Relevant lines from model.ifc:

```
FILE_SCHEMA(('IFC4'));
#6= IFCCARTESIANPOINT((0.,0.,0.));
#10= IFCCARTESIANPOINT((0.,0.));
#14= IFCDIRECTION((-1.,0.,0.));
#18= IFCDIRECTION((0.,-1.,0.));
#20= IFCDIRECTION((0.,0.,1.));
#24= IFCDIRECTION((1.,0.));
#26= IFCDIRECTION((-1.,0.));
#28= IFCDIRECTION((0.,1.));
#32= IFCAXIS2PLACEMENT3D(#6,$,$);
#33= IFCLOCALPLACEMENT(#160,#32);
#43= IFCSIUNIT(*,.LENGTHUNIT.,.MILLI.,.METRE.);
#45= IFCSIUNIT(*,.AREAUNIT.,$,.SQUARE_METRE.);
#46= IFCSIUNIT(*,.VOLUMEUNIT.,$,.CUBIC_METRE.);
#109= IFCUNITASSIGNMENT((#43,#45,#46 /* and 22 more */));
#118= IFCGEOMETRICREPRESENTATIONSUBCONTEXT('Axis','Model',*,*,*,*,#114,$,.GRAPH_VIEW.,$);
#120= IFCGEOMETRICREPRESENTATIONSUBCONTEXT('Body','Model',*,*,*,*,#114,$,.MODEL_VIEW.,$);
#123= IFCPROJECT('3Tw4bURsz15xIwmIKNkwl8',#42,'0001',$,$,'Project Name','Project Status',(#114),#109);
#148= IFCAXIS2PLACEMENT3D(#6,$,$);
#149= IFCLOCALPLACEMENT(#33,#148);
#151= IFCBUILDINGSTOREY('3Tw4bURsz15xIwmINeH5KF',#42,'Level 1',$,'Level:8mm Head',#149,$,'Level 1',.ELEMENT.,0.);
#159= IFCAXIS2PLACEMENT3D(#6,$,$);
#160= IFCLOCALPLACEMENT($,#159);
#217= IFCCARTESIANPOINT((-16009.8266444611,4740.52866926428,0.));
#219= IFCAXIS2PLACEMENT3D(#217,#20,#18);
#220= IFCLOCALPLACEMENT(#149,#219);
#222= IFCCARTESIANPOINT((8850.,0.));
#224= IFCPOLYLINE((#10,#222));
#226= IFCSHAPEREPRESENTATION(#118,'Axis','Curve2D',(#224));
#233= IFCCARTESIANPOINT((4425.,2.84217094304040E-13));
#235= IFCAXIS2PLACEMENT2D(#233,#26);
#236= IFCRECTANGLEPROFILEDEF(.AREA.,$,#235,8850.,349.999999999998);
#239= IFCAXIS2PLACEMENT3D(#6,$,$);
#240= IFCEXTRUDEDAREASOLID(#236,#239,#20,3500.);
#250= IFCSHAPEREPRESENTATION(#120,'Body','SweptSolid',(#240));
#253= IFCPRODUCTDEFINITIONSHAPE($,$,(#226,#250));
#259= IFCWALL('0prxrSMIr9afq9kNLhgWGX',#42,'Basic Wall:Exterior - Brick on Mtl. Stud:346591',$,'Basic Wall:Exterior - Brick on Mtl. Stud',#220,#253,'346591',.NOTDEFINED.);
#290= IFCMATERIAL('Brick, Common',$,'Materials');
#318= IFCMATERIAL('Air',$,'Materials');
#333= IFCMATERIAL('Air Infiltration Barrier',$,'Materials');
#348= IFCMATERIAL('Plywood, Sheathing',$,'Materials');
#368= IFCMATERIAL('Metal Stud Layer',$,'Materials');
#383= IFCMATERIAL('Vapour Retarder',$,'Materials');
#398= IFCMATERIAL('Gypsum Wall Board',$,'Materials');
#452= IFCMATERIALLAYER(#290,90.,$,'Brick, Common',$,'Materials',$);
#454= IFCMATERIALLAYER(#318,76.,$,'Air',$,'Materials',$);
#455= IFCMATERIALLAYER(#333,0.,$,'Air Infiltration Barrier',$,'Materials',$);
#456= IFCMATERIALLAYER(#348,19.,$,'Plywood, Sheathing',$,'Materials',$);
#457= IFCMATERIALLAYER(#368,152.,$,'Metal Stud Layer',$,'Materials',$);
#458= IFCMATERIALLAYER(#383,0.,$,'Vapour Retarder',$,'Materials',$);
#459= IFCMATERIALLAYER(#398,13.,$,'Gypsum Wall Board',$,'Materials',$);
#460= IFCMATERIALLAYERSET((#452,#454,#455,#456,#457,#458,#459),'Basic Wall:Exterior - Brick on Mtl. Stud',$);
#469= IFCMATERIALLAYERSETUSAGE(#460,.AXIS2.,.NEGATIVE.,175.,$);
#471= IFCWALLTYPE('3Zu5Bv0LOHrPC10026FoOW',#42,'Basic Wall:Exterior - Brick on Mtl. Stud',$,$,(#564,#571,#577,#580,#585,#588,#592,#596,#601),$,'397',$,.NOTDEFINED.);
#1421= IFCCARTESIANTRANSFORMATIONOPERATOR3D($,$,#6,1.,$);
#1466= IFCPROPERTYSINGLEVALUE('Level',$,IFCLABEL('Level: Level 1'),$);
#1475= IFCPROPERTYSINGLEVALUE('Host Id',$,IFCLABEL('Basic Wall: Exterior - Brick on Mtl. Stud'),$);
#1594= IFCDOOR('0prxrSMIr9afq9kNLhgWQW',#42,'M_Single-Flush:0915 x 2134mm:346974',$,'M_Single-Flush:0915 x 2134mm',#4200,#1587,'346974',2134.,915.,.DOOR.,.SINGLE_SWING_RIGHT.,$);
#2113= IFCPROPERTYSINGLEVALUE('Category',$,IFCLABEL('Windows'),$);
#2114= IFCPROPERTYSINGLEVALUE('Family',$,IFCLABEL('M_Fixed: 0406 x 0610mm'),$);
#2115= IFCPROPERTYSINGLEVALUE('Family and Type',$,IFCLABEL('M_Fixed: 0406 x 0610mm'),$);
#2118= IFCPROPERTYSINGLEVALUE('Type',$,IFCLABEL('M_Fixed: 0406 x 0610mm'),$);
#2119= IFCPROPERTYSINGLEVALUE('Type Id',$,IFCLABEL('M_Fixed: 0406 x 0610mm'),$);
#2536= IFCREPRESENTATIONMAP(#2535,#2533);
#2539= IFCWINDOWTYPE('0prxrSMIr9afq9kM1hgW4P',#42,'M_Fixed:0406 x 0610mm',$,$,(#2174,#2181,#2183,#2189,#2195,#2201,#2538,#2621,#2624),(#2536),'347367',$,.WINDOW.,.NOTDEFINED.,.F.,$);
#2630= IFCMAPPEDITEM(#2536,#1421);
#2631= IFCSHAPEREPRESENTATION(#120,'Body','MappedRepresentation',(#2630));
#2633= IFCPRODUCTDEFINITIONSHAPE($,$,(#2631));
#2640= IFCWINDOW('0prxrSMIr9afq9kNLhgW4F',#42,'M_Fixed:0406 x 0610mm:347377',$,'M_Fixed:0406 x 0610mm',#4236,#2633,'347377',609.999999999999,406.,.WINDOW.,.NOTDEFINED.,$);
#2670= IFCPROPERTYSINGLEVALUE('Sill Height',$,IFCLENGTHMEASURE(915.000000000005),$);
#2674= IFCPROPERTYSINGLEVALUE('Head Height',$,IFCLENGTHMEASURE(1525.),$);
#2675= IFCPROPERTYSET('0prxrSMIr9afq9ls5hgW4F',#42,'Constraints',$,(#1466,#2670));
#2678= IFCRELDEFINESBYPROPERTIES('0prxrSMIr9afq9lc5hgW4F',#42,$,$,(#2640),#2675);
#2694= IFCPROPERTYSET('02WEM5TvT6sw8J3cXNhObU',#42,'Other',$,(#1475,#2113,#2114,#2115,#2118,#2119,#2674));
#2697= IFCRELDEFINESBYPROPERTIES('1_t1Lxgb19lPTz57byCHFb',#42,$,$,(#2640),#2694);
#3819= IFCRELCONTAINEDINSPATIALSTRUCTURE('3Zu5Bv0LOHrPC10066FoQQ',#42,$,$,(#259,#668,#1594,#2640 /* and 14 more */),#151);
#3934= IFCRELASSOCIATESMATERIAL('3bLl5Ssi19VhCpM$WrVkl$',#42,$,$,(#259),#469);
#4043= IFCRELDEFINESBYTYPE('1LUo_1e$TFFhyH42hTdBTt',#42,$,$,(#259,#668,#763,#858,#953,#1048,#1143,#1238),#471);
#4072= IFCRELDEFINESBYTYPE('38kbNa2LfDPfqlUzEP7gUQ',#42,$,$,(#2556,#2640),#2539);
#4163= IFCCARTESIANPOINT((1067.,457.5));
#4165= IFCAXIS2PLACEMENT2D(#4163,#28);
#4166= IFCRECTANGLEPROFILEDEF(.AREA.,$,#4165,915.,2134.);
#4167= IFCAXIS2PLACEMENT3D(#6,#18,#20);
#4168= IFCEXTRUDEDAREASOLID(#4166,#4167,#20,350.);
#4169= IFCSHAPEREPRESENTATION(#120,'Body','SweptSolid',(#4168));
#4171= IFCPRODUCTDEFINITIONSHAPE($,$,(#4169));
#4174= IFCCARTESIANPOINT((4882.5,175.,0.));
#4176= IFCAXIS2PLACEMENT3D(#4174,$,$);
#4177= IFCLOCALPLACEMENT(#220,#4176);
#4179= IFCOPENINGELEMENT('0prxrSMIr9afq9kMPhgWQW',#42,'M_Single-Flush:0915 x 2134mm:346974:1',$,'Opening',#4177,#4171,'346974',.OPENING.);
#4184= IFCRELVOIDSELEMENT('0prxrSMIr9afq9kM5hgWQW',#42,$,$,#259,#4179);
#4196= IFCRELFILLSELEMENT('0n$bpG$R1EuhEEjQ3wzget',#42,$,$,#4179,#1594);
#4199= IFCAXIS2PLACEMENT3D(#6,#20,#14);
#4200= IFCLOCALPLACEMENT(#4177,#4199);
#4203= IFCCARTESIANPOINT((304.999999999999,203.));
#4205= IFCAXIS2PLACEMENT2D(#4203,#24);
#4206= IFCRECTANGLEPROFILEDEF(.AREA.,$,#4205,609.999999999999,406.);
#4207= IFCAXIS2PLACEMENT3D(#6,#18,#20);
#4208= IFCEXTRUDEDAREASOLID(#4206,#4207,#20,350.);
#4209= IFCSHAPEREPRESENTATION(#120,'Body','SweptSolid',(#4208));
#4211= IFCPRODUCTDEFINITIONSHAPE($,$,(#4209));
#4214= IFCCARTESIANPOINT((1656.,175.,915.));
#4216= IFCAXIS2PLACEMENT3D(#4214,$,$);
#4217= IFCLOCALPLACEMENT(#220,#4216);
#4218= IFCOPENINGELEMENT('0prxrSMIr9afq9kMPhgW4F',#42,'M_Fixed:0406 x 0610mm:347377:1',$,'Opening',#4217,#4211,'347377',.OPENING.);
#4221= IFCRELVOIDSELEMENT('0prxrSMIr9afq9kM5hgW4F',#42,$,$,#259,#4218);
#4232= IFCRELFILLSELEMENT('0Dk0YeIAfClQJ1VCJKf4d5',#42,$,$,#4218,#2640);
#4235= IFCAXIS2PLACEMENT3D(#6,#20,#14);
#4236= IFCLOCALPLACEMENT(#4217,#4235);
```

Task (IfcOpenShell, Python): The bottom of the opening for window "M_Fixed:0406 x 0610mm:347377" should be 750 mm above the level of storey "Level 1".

```python
import numpy as np
import ifcopenshell
import ifcopenshell.api.geometry
import ifcopenshell.api.pset
import ifcopenshell.geom
import ifcopenshell.util.element
import ifcopenshell.util.placement
import ifcopenshell.util.shape
import ifcopenshell.util.unit

model = ifcopenshell.open("model.ifc")
unit_scale = ifcopenshell.util.unit.calculate_unit_scale(model)

window = model.by_guid("0prxrSMIr9afq9kNLhgW4F")
opening = window.FillsVoids[0].RelatingOpeningElement
storey = ifcopenshell.util.element.get_container(window, ifc_class="IfcBuildingStorey")
level = ifcopenshell.util.placement.get_local_placement(storey.ObjectPlacement)[2, 3]

# The opening's origin need not be at the sill, so measure its lowest point.
shape = ifcopenshell.geom.create_shape(ifcopenshell.geom.settings(), opening)
bottom = ifcopenshell.util.shape.get_shape_bottom_elevation(shape, shape.geometry) / unit_scale
dz = level + 0.75 / unit_scale - bottom

shift = np.array([0.0, 0.0, dz])
# The window is placed relative to its opening, so it follows when the opening moves.
matrix = ifcopenshell.util.placement.get_local_placement(opening.ObjectPlacement)
matrix[:3, 3] += shift
ifcopenshell.api.geometry.edit_object_placement(
    model, product=opening, matrix=matrix, is_si=False, should_transform_children=True
)

# Keep the stored heights in step.
pset = model.by_id(ifcopenshell.util.element.get_pset(window, "Constraints", should_inherit=False)["id"])
ifcopenshell.api.pset.edit_pset(model, pset=pset, properties={
    "Sill Height": model.create_entity("IfcLengthMeasure", ifcopenshell.util.element.get_pset(window, "Constraints", "Sill Height") + dz),
})
pset = model.by_id(ifcopenshell.util.element.get_pset(window, "Other", should_inherit=False)["id"])
ifcopenshell.api.pset.edit_pset(model, pset=pset, properties={
    "Head Height": model.create_entity("IfcLengthMeasure", ifcopenshell.util.element.get_pset(window, "Other", "Head Height") + dz),
})

print(f"moved by {dz * unit_scale:+.3f} m")

model.write("model_rev.ifc")
```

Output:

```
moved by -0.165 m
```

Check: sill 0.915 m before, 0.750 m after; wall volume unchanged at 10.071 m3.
